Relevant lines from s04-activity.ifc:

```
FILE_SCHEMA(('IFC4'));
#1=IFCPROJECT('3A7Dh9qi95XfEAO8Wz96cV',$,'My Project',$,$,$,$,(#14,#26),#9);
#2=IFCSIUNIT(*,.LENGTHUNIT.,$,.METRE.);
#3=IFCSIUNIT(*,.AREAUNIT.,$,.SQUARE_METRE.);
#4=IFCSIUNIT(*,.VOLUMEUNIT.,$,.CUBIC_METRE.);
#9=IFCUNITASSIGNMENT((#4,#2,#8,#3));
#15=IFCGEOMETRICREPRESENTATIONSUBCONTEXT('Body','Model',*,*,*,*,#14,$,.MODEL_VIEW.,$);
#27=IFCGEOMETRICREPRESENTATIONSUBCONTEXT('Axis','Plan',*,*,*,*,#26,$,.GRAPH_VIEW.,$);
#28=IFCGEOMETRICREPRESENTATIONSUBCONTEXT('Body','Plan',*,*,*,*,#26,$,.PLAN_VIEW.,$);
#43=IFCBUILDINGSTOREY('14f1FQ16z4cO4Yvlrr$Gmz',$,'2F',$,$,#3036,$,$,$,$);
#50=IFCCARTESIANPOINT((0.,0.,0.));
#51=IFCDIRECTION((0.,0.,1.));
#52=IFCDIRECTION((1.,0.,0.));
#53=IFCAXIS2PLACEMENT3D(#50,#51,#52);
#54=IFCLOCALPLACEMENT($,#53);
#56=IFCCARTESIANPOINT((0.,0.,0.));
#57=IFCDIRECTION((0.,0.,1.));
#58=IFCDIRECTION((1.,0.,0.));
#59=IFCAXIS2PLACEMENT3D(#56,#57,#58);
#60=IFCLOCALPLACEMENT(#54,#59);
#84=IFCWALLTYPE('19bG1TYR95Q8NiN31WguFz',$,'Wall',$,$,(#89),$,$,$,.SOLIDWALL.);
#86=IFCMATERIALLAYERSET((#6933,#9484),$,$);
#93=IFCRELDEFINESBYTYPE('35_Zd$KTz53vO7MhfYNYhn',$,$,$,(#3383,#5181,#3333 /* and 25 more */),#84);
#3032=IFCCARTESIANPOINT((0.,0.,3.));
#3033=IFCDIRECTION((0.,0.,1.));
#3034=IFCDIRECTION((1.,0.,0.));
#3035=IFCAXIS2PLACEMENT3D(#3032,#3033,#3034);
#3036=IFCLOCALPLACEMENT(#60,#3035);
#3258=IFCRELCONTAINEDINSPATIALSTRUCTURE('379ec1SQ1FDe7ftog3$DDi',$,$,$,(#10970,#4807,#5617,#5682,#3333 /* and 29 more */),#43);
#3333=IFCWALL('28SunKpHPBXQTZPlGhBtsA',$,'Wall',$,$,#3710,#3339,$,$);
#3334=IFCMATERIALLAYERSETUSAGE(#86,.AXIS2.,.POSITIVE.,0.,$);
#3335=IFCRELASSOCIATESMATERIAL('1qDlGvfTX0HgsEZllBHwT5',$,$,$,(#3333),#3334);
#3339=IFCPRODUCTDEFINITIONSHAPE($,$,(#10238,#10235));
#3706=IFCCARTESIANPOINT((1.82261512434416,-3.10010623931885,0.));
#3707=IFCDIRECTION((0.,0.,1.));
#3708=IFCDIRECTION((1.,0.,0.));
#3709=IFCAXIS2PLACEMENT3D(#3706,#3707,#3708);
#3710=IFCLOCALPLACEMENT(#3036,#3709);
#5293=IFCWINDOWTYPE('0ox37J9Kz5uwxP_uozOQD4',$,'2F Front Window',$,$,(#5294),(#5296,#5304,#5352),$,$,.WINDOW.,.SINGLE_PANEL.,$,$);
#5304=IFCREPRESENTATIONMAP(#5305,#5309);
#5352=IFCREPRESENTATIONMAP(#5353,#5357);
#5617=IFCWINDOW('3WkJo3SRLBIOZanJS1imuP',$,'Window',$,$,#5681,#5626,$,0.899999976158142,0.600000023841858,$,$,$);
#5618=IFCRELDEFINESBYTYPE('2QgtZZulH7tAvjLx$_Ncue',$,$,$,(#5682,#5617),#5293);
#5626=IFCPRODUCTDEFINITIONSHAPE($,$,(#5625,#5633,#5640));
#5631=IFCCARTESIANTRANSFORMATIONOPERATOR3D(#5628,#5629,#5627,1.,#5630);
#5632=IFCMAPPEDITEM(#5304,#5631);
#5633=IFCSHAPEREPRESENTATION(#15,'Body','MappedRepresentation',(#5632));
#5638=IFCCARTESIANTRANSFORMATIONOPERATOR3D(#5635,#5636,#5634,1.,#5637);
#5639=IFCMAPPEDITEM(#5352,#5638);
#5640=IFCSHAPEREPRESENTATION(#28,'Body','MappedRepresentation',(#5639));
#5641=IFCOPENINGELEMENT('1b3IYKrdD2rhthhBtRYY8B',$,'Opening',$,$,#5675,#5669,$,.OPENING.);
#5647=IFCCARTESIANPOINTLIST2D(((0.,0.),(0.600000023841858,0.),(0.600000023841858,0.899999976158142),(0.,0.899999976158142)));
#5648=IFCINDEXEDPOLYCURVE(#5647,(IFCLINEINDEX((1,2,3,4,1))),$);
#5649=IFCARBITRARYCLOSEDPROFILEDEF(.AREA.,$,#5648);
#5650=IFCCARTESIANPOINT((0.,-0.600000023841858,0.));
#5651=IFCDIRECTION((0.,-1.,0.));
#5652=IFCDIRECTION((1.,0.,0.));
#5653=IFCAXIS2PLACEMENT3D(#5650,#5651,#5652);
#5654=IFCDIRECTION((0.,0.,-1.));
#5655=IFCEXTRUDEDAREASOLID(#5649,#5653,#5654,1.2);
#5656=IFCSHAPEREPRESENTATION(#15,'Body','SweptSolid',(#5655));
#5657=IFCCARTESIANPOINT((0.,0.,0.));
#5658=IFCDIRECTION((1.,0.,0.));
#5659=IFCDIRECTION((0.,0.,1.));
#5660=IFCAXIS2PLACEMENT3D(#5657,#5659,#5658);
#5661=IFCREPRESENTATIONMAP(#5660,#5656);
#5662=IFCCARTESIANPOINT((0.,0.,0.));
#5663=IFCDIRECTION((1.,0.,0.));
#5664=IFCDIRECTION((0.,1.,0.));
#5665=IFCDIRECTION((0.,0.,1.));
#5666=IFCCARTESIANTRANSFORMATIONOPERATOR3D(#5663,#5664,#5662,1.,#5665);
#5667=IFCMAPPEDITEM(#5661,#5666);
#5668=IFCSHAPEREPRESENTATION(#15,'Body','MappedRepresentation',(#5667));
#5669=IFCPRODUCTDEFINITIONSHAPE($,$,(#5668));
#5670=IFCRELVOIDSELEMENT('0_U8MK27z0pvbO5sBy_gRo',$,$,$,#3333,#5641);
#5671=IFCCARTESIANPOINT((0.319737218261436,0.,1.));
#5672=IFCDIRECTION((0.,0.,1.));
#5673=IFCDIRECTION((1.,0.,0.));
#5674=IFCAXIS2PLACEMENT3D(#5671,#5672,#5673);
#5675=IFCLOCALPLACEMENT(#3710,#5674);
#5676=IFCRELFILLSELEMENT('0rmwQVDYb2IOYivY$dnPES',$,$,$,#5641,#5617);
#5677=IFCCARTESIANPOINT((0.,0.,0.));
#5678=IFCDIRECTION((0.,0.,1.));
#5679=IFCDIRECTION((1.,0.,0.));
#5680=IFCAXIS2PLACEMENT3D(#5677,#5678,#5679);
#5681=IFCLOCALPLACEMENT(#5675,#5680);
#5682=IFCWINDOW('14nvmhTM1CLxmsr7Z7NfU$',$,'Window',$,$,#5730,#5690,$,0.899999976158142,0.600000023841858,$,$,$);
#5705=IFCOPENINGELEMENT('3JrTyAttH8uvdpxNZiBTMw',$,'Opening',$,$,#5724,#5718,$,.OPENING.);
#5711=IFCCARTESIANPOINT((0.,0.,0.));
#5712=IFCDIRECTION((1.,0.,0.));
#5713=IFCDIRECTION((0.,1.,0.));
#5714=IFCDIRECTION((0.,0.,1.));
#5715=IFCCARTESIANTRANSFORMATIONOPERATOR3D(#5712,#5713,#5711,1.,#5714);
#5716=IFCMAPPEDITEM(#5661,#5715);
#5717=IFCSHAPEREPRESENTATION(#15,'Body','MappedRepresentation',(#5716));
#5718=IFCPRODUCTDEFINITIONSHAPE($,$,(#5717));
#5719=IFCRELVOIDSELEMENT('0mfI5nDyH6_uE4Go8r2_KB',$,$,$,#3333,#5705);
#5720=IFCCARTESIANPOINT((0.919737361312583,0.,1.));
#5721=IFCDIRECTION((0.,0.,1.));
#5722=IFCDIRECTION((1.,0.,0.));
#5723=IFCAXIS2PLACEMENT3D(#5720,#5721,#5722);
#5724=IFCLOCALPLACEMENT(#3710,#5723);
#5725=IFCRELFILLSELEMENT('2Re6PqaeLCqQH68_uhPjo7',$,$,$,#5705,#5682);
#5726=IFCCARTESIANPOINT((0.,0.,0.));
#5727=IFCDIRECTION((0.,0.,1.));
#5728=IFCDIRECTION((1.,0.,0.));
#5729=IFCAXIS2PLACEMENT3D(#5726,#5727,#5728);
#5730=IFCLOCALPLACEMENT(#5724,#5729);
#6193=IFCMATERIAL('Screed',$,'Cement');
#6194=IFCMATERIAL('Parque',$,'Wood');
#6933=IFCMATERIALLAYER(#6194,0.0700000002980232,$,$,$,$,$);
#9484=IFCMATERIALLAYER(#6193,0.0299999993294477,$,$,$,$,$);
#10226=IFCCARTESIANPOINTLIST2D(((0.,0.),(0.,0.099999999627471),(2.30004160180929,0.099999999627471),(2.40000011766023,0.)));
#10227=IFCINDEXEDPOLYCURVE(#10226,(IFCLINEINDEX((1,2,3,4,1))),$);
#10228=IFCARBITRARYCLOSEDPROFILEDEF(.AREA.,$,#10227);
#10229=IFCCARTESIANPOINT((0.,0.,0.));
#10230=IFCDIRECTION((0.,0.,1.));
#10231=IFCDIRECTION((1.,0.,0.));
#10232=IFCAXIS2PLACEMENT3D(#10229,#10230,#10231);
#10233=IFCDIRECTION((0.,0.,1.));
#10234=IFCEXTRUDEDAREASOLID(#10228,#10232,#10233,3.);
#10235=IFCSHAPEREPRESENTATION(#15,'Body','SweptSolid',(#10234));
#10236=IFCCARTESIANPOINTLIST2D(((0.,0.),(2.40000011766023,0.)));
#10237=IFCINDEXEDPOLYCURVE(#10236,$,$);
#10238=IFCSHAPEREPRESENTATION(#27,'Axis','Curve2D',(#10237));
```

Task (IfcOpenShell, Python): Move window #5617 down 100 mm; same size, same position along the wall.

```python
import numpy as np
import ifcopenshell
import ifcopenshell.api.geometry
import ifcopenshell.util.placement
import ifcopenshell.util.unit

model = ifcopenshell.open("s04-activity.ifc")
unit_scale = ifcopenshell.util.unit.calculate_unit_scale(model)

window = model.by_guid("3WkJo3SRLBIOZanJS1imuP")
opening = window.FillsVoids[0].RelatingOpeningElement
dz = -0.1 / unit_scale

shift = np.array([0.0, 0.0, dz])
# The window is placed relative to its opening, so it follows when the opening moves.
matrix = ifcopenshell.util.placement.get_local_placement(opening.ObjectPlacement)
matrix[:3, 3] += shift
ifcopenshell.api.geometry.edit_object_placement(
    model, product=opening, matrix=matrix, is_si=False, should_transform_children=True
)

print(f"moved by {dz * unit_scale:+.3f} m")

model.write("s04-activity-out.ifc")
```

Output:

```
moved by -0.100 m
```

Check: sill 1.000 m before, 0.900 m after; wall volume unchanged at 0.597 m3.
